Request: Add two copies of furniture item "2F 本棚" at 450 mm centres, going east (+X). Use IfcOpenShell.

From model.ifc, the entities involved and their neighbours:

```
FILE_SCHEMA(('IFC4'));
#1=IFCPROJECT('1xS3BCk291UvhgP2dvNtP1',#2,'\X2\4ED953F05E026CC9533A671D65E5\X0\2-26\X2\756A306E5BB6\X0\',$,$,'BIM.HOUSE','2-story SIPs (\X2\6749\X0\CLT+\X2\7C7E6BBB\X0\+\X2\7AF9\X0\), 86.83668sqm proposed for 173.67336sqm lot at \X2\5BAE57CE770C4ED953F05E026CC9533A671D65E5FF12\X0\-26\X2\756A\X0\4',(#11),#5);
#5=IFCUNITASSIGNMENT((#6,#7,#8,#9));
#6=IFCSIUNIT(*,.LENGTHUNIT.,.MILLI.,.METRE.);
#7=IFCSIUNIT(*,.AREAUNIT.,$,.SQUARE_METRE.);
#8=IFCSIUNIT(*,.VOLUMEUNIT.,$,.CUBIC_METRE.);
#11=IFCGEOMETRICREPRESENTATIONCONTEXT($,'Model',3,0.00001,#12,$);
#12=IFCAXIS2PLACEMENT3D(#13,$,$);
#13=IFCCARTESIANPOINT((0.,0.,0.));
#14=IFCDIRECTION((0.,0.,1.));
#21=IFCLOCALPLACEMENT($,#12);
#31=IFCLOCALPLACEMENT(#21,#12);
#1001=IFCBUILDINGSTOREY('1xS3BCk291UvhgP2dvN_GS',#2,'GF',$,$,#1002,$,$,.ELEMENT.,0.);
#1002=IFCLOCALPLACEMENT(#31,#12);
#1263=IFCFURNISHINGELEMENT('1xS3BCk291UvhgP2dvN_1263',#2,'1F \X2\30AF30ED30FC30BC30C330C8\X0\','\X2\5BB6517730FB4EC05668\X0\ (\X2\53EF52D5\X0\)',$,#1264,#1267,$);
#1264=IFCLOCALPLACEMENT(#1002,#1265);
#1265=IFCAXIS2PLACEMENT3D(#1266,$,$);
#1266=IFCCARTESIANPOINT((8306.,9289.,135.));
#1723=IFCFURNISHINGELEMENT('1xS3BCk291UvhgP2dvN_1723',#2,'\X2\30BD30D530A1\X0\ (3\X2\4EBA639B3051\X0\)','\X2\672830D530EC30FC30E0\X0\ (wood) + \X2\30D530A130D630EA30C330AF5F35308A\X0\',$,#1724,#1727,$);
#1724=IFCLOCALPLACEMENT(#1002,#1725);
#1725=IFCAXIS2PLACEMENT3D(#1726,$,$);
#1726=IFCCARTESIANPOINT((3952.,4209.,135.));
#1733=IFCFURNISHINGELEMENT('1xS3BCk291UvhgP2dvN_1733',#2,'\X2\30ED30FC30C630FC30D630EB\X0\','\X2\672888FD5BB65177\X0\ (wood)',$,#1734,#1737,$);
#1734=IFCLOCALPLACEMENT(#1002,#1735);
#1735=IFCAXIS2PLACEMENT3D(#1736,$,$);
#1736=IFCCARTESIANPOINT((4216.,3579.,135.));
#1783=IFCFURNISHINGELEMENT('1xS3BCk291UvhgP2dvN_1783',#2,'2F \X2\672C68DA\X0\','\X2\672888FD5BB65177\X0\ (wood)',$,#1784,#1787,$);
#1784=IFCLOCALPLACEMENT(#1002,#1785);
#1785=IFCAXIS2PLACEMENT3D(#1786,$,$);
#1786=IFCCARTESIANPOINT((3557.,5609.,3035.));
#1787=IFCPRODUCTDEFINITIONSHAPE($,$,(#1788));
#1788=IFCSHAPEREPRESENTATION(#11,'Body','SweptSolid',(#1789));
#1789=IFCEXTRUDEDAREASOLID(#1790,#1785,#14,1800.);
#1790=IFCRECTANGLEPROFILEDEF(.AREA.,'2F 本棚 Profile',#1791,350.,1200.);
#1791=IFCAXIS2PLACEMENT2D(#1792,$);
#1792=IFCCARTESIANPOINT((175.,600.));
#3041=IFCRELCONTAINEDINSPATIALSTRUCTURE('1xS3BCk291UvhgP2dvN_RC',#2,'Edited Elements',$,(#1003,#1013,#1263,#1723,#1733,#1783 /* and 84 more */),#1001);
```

```python
import numpy as np
import ifcopenshell
import ifcopenshell.api.geometry
import ifcopenshell.api.root
import ifcopenshell.util.element
import ifcopenshell.util.placement
import ifcopenshell.util.unit

model = ifcopenshell.open("model.ifc")
unit_scale = ifcopenshell.util.unit.calculate_unit_scale(model)


def reuse_history(source, copy):
    """copy_class also copies each property set's owner history, people and application; keep the originals."""
    for rel in copy.IsDefinedBy:
        if rel.is_a("IfcRelDefinesByProperties") and (history := rel.RelatingPropertyDefinition.OwnerHistory):
            rel.RelatingPropertyDefinition.OwnerHistory = source.OwnerHistory
            ifcopenshell.util.element.remove_deep2(model, history)


source = model.by_guid("1xS3BCk291UvhgP2dvN_1783")
base = ifcopenshell.util.placement.get_local_placement(source.ObjectPlacement)
step = np.array([1.0, 0.0, 0.0]) * 0.45 / unit_scale

for i in range(1, 3):
    copy = ifcopenshell.api.root.copy_class(model, product=source)
    copy.Representation = ifcopenshell.util.element.copy_deep(
        model, source.Representation, exclude=["IfcGeometricRepresentationContext", "IfcRepresentationMap"]
    )
    reuse_history(source, copy)
    matrix = base.copy()
    matrix[:3, 3] += i * step
    print("added at", matrix[:3, 3].round(3) + 0.0)
    ifcopenshell.api.geometry.edit_object_placement(model, product=copy, matrix=matrix, is_si=False)

model.write("model_rev.ifc")
```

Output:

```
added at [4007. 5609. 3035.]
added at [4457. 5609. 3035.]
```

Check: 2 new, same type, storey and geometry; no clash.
